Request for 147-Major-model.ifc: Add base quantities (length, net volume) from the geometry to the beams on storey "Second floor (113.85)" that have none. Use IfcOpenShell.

First a look at what the model holds.

```python
import ifcopenshell
import ifcopenshell.util.element
import ifcopenshell.util.unit

model = ifcopenshell.open("147-Major-model.ifc")
print(model.schema)
for unit_type in ("LENGTHUNIT", "AREAUNIT", "VOLUMEUNIT"):
    print(unit_type, ifcopenshell.util.unit.calculate_unit_scale(model, unit_type))
storey = next(s for s in model.by_type("IfcBuildingStorey") if s.Name == "Second floor (113.85)")
beams = [e for e in ifcopenshell.util.element.get_decomposition(storey) if e.is_a("IfcBeam")]
for e in sorted(beams, key=lambda e: e.id()):
    print(e.id(), e.is_a(), e.Name, list(ifcopenshell.util.element.get_psets(e, qtos_only=True)), sep=" | ")
```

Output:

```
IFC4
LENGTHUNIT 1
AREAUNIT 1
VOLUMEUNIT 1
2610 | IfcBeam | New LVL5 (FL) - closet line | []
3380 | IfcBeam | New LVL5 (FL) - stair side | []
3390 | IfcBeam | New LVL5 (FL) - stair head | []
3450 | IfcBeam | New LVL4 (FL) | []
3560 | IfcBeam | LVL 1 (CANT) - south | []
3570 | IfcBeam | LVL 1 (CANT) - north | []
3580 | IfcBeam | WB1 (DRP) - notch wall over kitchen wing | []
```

```python
import ifcopenshell
import ifcopenshell.api.pset
import ifcopenshell.geom
import ifcopenshell.util.element
import ifcopenshell.util.shape
import ifcopenshell.util.unit

model = ifcopenshell.open("147-Major-model.ifc")
unit_scale = ifcopenshell.util.unit.calculate_unit_scale(model)
volume_scale = ifcopenshell.util.unit.calculate_unit_scale(model, "VOLUMEUNIT")
settings = ifcopenshell.geom.settings()

storey = next(s for s in model.by_type("IfcBuildingStorey") if s.Name == "Second floor (113.85)")
beams = [e for e in ifcopenshell.util.element.get_decomposition(storey) if e.is_a("IfcBeam")]

for e in sorted(beams, key=lambda e: e.id()):
    if ifcopenshell.util.element.get_psets(e, qtos_only=True, should_inherit=False):
        continue
    # Geometry comes back in metres, in the element's own axes.
    shape = ifcopenshell.geom.create_shape(settings, e)
    values = {
        "Length": ifcopenshell.util.shape.get_max_xyz(shape.geometry) / unit_scale,
        "NetVolume": ifcopenshell.util.shape.get_volume(shape.geometry) / volume_scale,
    }
    qto = ifcopenshell.api.pset.add_qto(model, product=e, name="Qto_BeamBaseQuantities")
    ifcopenshell.api.pset.edit_qto(model, qto=qto, properties=values)
    print(e.id(), {k: round(v, 3) for k, v in values.items()})

model.write("147-Major-model_v2.ifc")
```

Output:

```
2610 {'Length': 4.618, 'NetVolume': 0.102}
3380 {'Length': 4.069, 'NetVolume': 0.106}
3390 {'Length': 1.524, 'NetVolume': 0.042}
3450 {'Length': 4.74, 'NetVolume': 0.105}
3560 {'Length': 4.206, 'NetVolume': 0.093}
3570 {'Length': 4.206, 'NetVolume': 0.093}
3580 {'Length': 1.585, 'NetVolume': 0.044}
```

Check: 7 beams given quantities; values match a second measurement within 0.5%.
